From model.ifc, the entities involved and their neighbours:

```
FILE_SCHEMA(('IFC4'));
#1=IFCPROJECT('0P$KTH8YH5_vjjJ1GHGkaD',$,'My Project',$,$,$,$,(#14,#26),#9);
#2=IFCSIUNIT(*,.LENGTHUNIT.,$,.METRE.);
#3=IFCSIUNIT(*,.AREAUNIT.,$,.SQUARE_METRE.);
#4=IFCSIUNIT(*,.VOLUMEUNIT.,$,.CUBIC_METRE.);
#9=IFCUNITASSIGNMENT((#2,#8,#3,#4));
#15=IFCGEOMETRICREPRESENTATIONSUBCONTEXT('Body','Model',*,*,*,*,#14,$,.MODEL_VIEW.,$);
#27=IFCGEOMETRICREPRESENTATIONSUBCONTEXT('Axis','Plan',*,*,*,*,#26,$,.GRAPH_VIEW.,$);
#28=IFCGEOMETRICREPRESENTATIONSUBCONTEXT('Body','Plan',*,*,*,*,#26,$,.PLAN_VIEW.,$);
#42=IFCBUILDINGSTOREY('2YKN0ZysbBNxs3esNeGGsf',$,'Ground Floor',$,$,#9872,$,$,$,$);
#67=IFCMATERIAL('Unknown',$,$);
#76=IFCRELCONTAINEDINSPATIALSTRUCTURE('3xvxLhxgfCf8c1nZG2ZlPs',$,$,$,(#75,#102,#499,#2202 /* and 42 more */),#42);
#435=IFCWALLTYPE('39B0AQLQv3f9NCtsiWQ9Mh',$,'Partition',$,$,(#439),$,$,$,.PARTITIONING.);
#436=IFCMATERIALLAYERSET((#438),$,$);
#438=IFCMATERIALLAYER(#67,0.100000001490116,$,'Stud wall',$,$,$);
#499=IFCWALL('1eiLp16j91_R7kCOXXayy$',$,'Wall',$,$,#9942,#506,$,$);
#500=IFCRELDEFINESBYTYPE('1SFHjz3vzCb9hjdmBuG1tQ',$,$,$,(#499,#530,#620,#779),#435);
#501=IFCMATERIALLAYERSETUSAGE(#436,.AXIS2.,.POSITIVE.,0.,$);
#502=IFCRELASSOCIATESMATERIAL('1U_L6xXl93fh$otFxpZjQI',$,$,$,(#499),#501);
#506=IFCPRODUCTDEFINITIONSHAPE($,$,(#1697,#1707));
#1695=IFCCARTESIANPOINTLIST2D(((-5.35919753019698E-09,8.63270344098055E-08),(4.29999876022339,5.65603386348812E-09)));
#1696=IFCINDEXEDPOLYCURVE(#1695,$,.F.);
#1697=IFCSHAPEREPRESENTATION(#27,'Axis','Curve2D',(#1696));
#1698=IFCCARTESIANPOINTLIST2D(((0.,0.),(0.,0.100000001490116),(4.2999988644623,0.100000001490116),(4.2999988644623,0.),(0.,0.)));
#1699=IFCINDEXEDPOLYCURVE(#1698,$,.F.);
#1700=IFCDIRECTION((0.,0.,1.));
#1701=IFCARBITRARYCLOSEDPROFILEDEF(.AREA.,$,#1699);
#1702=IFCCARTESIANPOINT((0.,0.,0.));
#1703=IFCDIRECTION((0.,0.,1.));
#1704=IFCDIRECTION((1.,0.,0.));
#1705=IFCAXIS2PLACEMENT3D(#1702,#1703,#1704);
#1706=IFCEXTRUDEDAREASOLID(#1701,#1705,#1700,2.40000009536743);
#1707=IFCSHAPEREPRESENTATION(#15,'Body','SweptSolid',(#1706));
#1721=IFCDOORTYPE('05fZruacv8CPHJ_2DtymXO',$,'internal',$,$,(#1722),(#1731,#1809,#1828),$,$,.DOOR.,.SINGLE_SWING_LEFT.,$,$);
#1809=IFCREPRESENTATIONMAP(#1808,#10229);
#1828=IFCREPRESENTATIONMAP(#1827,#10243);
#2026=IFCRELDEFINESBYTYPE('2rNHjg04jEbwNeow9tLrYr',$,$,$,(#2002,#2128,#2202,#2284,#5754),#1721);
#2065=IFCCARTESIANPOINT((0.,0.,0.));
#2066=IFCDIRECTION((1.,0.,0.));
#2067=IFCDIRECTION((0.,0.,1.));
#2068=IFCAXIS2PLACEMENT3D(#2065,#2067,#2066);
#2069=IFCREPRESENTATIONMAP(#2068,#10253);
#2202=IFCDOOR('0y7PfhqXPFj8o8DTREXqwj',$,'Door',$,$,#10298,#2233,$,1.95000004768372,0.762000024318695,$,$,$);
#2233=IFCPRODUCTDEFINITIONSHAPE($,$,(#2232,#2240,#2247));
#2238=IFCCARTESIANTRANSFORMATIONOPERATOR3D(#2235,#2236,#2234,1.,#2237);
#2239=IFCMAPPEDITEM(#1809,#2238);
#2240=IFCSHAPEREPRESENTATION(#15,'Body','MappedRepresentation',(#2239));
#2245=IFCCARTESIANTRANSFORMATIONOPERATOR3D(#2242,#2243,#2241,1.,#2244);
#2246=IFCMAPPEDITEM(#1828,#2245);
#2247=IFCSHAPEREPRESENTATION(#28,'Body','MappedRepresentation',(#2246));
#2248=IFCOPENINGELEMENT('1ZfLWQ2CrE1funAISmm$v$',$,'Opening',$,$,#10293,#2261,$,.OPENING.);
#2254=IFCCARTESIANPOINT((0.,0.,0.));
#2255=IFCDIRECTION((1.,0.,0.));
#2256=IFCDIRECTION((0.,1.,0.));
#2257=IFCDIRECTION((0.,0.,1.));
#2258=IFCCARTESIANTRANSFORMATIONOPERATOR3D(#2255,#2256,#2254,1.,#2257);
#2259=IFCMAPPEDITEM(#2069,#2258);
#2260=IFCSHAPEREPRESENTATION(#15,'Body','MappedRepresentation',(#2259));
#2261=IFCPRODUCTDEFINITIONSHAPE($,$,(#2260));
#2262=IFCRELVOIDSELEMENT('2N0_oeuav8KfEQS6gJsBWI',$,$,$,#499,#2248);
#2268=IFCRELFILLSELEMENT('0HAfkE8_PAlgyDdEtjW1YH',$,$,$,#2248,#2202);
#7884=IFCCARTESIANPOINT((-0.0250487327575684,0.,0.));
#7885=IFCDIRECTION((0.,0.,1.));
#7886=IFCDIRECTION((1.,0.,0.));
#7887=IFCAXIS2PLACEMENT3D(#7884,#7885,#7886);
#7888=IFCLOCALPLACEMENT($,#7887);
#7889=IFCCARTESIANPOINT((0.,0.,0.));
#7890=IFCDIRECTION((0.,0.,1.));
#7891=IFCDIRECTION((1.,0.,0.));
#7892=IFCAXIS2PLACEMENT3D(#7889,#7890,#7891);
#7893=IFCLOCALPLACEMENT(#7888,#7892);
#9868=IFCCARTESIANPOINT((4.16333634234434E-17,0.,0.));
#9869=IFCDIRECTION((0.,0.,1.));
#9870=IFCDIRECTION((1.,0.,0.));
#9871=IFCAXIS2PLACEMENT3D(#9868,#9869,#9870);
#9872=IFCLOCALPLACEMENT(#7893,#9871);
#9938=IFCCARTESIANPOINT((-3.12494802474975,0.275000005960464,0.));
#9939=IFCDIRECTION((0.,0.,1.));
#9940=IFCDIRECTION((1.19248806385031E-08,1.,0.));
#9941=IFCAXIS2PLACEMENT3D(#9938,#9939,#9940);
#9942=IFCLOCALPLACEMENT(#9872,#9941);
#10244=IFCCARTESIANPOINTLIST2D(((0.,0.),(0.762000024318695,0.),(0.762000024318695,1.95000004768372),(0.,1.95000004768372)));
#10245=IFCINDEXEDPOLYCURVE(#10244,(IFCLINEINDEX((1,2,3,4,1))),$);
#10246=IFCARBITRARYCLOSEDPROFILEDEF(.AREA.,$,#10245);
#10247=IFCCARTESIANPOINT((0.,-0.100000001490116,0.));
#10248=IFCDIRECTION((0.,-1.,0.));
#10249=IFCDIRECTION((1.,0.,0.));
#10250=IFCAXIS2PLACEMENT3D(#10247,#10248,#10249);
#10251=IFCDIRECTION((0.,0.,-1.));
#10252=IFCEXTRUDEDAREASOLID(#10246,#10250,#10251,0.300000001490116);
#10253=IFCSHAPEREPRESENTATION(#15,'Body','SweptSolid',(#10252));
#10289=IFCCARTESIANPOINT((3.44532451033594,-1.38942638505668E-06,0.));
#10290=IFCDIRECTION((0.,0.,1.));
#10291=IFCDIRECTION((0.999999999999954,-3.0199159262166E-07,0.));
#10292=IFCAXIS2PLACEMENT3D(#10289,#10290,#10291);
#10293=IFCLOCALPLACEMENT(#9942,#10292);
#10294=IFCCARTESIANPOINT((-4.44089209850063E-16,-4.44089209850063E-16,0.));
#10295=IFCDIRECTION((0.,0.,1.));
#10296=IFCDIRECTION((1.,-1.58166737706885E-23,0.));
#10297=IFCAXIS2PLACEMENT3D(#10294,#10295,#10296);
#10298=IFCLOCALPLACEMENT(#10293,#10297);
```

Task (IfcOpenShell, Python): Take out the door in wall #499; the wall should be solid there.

```python
import ifcopenshell
import ifcopenshell.api.feature
import ifcopenshell.api.root
import ifcopenshell.geom
import ifcopenshell.util.shape

model = ifcopenshell.open("model.ifc")
settings = ifcopenshell.geom.settings()


def volume(element):
    """Net volume in cubic metres, openings subtracted."""
    shape = ifcopenshell.geom.create_shape(settings, element)
    return ifcopenshell.util.shape.get_volume(shape.geometry)


door = model.by_id(2202)
opening = door.FillsVoids[0].RelatingOpeningElement
wall = opening.VoidsElements[0].RelatingBuildingElement
before = volume(wall)

ifcopenshell.api.root.remove_product(model, product=door)
ifcopenshell.api.feature.remove_feature(model, feature=opening)

after = volume(wall)

print(f"wall volume {before:.3f} -> {after:.3f} m3")

model.write("model_rev.ifc")
```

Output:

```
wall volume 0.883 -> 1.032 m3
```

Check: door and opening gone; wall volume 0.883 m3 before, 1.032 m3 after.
